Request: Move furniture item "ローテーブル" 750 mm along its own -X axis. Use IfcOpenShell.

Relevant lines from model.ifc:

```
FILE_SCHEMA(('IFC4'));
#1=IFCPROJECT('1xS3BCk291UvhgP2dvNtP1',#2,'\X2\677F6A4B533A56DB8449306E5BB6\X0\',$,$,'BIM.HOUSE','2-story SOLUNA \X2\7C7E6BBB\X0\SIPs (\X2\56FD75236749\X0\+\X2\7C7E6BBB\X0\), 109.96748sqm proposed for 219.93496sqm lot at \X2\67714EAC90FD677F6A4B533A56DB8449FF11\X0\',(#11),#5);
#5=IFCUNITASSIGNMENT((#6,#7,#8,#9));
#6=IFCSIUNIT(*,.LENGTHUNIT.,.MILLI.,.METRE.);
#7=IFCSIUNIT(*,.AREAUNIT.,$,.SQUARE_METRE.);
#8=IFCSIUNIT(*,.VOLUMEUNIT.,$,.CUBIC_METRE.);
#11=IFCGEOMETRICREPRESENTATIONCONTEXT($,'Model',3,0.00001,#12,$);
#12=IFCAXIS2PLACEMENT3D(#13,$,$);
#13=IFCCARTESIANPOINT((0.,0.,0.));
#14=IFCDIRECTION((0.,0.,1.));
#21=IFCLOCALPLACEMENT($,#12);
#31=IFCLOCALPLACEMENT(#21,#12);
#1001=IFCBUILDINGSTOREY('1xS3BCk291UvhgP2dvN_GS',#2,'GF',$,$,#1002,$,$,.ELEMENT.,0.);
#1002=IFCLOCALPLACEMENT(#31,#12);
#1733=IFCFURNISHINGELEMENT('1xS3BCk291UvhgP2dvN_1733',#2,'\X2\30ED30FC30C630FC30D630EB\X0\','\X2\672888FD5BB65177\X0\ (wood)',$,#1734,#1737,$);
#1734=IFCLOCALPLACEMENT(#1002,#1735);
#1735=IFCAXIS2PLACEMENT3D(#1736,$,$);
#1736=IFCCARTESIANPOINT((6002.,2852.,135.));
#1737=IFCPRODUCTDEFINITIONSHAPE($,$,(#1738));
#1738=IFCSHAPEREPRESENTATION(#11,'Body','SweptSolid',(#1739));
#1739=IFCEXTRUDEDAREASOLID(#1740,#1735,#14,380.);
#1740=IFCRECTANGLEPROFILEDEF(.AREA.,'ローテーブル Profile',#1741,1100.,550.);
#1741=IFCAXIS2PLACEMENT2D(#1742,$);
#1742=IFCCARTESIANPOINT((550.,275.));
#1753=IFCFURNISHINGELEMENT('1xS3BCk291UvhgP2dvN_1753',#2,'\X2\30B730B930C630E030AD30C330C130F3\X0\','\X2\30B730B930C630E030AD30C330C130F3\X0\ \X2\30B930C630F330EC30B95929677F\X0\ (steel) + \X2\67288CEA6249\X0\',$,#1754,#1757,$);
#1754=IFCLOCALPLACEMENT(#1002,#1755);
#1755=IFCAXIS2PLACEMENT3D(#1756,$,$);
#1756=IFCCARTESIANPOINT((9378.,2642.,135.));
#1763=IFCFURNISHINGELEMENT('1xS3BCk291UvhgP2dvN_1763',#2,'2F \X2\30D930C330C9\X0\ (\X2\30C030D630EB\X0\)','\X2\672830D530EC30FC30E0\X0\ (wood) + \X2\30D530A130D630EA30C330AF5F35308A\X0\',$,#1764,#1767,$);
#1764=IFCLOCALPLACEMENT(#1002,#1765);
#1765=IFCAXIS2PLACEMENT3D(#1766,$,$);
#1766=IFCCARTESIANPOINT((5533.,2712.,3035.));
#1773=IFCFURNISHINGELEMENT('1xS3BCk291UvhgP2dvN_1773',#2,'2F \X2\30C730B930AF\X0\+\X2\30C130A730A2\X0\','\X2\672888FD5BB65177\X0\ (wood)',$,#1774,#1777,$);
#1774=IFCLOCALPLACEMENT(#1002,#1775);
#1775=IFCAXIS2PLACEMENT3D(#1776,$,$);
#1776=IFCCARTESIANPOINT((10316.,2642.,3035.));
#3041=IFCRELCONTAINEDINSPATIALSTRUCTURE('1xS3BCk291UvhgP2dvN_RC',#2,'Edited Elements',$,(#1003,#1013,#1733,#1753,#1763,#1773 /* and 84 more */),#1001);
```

```python
import ifcopenshell
import ifcopenshell.api.geometry
import ifcopenshell.util.placement
import ifcopenshell.util.unit

model = ifcopenshell.open("model.ifc")
unit_scale = ifcopenshell.util.unit.calculate_unit_scale(model)

item = model.by_id(1733)
matrix = ifcopenshell.util.placement.get_local_placement(item.ObjectPlacement)
matrix[:3, 3] -= matrix[:3, 0] * 0.75 / unit_scale
ifcopenshell.api.geometry.edit_object_placement(model, product=item, matrix=matrix, is_si=False)

print(ifcopenshell.util.placement.get_local_placement(item.ObjectPlacement).round(3) + 0.0)

model.write("model_v2.ifc")
```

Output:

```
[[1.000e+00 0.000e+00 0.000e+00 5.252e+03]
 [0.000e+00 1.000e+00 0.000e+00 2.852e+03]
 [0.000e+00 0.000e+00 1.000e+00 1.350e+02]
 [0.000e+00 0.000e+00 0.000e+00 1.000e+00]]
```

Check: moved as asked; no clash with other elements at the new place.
